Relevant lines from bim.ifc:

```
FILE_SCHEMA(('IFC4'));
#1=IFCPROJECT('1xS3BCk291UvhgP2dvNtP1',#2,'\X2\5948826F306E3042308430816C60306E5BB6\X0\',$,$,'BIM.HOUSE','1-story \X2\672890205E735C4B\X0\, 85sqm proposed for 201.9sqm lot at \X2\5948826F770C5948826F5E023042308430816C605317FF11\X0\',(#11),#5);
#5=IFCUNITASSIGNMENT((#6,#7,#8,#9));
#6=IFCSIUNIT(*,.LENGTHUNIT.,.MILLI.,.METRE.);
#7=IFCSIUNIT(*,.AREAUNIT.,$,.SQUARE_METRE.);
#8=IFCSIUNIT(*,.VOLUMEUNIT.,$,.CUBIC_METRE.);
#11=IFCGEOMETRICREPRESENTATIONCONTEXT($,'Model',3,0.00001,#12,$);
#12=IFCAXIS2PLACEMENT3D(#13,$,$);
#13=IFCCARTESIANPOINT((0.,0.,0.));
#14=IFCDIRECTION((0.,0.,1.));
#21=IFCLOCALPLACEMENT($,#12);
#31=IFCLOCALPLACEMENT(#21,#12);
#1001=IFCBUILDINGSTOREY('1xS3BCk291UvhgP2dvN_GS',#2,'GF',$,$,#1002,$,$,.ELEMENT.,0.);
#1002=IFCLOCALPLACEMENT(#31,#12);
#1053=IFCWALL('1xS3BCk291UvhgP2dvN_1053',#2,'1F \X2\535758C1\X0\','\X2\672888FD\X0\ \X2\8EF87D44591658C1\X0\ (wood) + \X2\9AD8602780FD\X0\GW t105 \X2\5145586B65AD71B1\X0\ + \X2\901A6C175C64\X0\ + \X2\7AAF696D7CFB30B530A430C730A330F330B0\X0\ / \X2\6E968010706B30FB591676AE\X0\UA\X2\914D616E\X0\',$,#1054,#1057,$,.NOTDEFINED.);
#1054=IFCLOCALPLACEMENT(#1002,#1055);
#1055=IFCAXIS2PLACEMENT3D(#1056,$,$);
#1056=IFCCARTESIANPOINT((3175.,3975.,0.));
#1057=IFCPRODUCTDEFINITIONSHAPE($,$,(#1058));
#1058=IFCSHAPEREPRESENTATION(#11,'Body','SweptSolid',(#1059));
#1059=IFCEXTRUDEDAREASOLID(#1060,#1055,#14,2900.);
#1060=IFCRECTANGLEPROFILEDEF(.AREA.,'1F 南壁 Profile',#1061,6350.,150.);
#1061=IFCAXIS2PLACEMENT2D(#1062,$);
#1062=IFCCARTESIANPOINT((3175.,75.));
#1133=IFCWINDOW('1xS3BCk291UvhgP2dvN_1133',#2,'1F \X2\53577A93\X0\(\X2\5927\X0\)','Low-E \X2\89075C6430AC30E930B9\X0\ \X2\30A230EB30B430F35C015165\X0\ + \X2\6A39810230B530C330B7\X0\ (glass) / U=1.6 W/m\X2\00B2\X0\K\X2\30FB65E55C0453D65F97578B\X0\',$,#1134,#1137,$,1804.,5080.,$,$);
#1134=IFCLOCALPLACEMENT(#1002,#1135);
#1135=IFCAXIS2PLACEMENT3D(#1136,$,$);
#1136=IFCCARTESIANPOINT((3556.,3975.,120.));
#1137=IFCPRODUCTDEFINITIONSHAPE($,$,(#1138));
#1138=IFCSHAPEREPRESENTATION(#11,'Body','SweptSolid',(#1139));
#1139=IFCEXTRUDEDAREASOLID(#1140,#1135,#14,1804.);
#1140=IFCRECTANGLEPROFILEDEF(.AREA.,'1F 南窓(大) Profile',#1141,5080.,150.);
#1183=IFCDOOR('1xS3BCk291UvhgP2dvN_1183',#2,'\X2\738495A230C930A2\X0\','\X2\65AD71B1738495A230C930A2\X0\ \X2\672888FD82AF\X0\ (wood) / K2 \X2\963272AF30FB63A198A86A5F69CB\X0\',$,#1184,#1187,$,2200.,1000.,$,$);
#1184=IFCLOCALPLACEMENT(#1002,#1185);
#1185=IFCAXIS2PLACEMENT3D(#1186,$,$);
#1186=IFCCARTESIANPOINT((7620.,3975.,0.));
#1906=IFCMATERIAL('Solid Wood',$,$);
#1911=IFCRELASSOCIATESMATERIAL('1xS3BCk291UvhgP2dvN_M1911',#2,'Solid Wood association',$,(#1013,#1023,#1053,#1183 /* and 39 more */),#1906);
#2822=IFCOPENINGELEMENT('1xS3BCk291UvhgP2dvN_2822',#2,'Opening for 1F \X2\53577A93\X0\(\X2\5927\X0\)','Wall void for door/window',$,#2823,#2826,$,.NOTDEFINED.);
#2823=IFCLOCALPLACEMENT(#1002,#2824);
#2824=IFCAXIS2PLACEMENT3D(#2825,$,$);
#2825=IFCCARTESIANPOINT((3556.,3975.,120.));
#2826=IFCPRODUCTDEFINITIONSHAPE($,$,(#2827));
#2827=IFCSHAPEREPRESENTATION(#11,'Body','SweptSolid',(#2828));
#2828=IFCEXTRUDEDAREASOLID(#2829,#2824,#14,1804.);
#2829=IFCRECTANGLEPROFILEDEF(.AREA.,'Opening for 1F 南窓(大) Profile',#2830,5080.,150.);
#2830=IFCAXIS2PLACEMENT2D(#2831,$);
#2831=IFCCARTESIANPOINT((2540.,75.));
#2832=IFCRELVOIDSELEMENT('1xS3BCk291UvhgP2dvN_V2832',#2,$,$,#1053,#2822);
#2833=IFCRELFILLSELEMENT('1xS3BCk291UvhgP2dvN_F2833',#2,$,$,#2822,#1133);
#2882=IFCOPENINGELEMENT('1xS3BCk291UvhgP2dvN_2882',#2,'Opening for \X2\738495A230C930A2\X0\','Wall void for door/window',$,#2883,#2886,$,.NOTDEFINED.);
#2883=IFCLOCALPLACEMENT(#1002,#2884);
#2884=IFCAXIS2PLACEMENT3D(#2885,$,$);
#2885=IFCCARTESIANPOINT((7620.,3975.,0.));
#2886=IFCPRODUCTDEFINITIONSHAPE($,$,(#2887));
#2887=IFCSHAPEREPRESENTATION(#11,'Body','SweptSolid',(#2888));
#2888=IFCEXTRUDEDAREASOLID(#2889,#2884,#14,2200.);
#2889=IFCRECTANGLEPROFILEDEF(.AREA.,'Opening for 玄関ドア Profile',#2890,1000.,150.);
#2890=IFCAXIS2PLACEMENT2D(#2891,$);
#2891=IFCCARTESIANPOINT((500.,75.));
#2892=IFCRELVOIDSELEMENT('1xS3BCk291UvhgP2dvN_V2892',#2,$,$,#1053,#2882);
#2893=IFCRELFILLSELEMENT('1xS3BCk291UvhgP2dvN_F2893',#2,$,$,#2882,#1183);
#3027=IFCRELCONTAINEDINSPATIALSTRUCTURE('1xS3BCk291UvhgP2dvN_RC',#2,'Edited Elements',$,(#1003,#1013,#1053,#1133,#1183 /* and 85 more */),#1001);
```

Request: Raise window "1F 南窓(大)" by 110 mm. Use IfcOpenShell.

```python
import numpy as np
import ifcopenshell
import ifcopenshell.api.geometry
import ifcopenshell.util.placement
import ifcopenshell.util.unit

model = ifcopenshell.open("bim.ifc")
unit_scale = ifcopenshell.util.unit.calculate_unit_scale(model)

window = model.by_guid("1xS3BCk291UvhgP2dvN_1133")
opening = window.FillsVoids[0].RelatingOpeningElement
dz = 0.11 / unit_scale

shift = np.array([0.0, 0.0, dz])
# The window is not placed relative to its opening, so move both.
for product in (opening, window):
    matrix = ifcopenshell.util.placement.get_local_placement(product.ObjectPlacement)
    matrix[:3, 3] += shift
    ifcopenshell.api.geometry.edit_object_placement(model, product=product, matrix=matrix, is_si=False)

print(f"moved by {dz * unit_scale:+.3f} m")

model.write("bim_v2.ifc")
```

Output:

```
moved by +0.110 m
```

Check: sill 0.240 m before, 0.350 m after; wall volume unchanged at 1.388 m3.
